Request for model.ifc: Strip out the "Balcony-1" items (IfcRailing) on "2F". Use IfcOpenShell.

First a look at what the model holds.

```python
import ifcopenshell
import ifcopenshell.util.element

model = ifcopenshell.open("model.ifc")
print(model.schema)
storey = next(s for s in model.by_type("IfcBuildingStorey") if s.Name == "2F")
railings = [e for e in ifcopenshell.util.element.get_decomposition(storey) if e.is_a("IfcRailing")]
seen = {}
for e in railings:
    element_type = ifcopenshell.util.element.get_type(e)
    name = element_type.Name if element_type not in (None, e) else None
    seen[name] = seen.get(name, 0) + 1
for name, count in sorted(seen.items(), key=str):
    print(count, "x", name)
```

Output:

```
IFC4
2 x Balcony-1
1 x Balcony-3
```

```python
import ifcopenshell
import ifcopenshell.api.root
import ifcopenshell.util.element

model = ifcopenshell.open("model.ifc")

storey = next(s for s in model.by_type("IfcBuildingStorey") if s.Name == "2F")
railings = [e for e in ifcopenshell.util.element.get_decomposition(storey) if e.is_a("IfcRailing")]
targets = [e for e in railings if (t := ifcopenshell.util.element.get_type(e)) not in (None, e) and t.Name == "Balcony-1"]

for e in targets:
    ifcopenshell.api.root.remove_product(model, product=e)
print(len(targets), "removed")

model.write("model_edited.ifc")
```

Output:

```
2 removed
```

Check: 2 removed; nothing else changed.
